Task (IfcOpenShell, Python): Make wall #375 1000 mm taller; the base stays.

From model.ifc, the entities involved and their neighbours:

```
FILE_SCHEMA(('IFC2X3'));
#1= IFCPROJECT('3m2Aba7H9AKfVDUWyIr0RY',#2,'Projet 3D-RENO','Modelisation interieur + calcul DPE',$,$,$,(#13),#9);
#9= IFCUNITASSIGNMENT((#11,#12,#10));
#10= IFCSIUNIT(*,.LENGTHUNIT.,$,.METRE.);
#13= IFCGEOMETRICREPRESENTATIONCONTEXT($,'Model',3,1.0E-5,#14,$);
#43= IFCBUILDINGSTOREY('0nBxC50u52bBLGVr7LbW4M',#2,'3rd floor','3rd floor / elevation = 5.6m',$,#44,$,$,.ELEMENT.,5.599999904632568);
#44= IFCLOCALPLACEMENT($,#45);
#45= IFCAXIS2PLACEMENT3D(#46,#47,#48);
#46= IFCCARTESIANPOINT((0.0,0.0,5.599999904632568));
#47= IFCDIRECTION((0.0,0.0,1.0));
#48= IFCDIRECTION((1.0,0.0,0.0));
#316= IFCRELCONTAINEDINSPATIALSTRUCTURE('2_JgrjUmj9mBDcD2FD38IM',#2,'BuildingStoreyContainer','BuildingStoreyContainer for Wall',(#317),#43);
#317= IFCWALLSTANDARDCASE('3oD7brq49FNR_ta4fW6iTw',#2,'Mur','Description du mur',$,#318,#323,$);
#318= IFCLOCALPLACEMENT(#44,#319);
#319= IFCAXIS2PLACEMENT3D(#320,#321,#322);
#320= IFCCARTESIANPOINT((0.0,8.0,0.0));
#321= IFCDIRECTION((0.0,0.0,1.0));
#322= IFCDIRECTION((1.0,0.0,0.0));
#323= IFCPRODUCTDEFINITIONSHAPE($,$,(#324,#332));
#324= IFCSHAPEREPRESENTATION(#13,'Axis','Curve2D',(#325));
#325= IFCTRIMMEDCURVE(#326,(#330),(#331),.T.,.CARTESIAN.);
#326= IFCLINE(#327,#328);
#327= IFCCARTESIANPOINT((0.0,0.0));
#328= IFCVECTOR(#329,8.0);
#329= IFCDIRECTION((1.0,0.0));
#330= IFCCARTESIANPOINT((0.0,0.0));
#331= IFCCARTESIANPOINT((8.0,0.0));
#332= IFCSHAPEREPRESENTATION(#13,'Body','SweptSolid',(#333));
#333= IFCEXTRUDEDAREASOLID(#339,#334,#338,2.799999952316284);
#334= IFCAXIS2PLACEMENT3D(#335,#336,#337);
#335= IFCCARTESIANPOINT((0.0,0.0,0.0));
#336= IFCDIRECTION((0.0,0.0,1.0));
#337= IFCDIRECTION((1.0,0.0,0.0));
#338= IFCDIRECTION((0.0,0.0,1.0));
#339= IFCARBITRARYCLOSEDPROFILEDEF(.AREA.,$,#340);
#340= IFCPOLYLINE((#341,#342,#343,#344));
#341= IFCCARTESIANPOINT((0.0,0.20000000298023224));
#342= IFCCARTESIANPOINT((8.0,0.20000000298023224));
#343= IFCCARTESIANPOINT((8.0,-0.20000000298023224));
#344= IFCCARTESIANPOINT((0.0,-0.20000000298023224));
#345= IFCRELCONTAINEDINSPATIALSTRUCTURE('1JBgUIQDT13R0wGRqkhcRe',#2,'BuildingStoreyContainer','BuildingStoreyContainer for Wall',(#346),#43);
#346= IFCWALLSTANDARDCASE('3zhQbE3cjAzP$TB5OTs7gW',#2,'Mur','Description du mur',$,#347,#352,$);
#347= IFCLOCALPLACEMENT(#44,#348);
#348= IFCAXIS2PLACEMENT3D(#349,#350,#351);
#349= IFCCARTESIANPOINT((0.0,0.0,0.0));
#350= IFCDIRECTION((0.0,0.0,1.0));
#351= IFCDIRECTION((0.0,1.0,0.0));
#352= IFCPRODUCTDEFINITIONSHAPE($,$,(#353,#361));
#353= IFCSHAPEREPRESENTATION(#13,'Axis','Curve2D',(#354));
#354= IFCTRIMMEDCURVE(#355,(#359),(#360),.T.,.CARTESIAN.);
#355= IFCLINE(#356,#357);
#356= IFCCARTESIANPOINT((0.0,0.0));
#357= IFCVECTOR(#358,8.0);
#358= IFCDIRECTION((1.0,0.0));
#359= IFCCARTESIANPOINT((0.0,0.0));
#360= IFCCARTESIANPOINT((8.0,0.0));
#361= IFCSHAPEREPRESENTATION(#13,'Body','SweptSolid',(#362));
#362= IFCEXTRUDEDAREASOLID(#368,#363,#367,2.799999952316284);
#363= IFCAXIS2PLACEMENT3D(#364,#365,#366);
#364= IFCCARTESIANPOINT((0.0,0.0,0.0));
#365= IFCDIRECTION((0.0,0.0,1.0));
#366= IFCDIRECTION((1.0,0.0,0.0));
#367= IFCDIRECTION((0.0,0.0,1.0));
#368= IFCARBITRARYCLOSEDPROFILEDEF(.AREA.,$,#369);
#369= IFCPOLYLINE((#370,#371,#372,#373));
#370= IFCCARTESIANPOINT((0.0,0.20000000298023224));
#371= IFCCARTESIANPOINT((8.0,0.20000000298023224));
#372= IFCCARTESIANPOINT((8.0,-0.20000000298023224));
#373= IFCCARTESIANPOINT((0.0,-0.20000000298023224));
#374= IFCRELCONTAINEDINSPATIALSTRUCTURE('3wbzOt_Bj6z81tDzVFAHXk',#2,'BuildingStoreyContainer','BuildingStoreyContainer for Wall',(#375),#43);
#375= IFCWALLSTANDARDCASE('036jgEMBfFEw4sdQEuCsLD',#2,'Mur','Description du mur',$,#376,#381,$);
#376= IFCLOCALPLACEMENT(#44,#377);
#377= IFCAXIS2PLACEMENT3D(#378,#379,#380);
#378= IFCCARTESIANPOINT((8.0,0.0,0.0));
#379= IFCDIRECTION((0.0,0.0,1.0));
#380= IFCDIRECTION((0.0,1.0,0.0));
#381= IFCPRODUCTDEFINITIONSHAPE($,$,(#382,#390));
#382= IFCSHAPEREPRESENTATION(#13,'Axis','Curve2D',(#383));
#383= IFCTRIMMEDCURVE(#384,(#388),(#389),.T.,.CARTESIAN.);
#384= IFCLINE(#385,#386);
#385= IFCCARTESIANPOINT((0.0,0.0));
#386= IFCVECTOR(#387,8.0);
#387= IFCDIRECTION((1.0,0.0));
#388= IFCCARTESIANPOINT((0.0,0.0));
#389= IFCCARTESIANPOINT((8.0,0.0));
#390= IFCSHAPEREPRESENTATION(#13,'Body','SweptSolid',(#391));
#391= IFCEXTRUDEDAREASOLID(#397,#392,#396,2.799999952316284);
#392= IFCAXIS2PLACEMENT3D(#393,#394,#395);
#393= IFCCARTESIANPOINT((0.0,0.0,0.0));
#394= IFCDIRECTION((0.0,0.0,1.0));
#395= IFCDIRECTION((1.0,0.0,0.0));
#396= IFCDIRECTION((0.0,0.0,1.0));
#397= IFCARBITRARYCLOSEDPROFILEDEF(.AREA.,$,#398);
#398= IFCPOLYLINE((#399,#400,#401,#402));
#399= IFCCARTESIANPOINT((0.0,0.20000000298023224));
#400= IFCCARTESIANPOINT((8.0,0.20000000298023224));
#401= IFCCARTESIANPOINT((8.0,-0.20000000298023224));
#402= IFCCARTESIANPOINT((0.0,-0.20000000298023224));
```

```python
import ifcopenshell
import ifcopenshell.geom
import ifcopenshell.util.shape
import ifcopenshell.util.unit

model = ifcopenshell.open("model.ifc")
unit_scale = ifcopenshell.util.unit.calculate_unit_scale(model)
settings = ifcopenshell.geom.settings()


def volume(element):
    """Net volume in cubic metres, openings subtracted."""
    shape = ifcopenshell.geom.create_shape(settings, element)
    return ifcopenshell.util.shape.get_volume(shape.geometry)


wall = model.by_guid("036jgEMBfFEw4sdQEuCsLD")
before = volume(wall)

body = next(r for r in wall.Representation.Representations if r.RepresentationIdentifier == "Body")
solid = body.Items[0]
old_height = solid.Depth
solid.Depth += 1 / unit_scale
after = volume(wall)

print(f"height {old_height:g} -> {solid.Depth:g}, volume {before:.3f} -> {after:.3f} m3")

model.write("model_edited.ifc")
```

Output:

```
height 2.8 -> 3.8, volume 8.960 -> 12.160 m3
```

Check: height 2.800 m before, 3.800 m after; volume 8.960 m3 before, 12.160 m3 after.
